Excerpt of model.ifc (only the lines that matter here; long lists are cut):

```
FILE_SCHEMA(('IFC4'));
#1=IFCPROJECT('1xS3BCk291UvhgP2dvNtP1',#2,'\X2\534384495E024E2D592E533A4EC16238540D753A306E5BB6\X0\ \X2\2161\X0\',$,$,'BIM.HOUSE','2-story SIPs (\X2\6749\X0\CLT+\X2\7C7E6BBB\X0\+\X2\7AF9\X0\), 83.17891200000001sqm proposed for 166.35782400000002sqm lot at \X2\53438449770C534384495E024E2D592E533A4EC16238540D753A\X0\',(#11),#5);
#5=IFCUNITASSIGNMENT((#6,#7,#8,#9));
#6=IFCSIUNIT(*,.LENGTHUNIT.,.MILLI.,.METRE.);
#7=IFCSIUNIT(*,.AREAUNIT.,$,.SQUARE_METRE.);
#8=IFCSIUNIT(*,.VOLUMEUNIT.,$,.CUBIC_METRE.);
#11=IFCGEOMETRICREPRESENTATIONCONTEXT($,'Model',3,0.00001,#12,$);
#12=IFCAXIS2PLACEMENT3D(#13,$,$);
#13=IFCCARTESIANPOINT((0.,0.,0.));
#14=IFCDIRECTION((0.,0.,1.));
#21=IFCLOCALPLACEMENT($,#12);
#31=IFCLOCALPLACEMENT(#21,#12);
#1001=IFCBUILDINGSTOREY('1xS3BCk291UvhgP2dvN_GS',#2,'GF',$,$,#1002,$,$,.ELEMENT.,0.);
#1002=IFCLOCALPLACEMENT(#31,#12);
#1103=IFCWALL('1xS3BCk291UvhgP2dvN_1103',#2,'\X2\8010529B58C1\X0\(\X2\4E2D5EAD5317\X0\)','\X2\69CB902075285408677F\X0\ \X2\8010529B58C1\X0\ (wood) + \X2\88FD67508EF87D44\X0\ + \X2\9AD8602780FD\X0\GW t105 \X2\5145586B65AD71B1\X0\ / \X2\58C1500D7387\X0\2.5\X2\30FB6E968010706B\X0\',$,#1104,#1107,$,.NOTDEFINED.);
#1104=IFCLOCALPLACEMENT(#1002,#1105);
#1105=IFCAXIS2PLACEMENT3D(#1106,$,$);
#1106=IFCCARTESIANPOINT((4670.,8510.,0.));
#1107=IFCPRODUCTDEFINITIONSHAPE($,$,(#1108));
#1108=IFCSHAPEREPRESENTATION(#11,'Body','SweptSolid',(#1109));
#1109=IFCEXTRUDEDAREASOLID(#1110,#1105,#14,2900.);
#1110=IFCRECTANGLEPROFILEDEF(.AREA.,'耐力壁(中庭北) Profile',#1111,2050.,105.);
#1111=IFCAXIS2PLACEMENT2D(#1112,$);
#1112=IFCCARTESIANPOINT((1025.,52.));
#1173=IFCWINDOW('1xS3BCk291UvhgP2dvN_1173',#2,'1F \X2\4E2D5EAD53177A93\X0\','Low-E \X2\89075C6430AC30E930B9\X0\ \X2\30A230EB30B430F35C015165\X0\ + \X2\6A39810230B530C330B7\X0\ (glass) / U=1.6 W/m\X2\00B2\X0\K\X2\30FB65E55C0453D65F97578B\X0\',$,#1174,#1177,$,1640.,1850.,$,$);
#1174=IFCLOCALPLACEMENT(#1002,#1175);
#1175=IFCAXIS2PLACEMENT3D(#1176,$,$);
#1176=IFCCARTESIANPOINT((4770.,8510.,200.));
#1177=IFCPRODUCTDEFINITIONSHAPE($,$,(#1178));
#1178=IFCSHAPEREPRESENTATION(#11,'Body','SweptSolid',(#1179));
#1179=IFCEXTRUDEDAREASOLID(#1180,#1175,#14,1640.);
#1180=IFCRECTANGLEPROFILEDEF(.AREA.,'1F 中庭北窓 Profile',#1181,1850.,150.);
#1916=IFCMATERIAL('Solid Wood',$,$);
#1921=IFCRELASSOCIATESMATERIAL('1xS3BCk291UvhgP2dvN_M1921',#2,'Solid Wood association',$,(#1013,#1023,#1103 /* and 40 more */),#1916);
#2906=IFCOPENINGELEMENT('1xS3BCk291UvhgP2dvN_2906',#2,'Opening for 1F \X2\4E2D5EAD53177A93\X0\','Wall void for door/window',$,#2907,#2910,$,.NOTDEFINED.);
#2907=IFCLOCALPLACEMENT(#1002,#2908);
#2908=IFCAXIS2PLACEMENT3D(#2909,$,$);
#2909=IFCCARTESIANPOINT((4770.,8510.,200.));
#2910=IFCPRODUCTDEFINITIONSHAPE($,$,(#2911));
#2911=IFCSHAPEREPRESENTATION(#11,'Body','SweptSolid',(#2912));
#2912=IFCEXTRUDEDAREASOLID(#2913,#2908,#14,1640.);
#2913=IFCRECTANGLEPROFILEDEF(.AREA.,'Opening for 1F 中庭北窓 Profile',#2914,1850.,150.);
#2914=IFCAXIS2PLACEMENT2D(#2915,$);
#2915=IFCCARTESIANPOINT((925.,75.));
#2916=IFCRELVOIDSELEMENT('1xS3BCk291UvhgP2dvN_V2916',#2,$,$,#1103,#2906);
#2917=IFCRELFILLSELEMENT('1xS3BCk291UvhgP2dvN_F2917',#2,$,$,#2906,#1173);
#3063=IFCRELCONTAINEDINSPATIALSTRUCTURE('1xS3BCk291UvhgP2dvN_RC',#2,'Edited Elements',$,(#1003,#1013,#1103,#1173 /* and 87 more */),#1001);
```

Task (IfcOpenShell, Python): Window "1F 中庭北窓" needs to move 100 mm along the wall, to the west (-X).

```python
import ifcopenshell
import ifcopenshell.api.geometry
import ifcopenshell.util.placement

model = ifcopenshell.open("model.ifc")

window = model.by_guid("1xS3BCk291UvhgP2dvN_1173")
opening = window.FillsVoids[0].RelatingOpeningElement
wall = opening.VoidsElements[0].RelatingBuildingElement

wall_matrix = ifcopenshell.util.placement.get_local_placement(wall.ObjectPlacement)
shift = wall_matrix[:3, 0] * -100.0
before = ifcopenshell.util.placement.get_local_placement(window.ObjectPlacement)[:3, 3].copy()

# The window is not placed relative to its opening, so move both.
for product in (opening, window):
    matrix = ifcopenshell.util.placement.get_local_placement(product.ObjectPlacement)
    matrix[:3, 3] += shift
    ifcopenshell.api.geometry.edit_object_placement(model, product=product, matrix=matrix, is_si=False)

after = ifcopenshell.util.placement.get_local_placement(window.ObjectPlacement)[:3, 3]
print("window moved by", (after - before).round(3) + 0.0)

model.write("model_rev.ifc")
```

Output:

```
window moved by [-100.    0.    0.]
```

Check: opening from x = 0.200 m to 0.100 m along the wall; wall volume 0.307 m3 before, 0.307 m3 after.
